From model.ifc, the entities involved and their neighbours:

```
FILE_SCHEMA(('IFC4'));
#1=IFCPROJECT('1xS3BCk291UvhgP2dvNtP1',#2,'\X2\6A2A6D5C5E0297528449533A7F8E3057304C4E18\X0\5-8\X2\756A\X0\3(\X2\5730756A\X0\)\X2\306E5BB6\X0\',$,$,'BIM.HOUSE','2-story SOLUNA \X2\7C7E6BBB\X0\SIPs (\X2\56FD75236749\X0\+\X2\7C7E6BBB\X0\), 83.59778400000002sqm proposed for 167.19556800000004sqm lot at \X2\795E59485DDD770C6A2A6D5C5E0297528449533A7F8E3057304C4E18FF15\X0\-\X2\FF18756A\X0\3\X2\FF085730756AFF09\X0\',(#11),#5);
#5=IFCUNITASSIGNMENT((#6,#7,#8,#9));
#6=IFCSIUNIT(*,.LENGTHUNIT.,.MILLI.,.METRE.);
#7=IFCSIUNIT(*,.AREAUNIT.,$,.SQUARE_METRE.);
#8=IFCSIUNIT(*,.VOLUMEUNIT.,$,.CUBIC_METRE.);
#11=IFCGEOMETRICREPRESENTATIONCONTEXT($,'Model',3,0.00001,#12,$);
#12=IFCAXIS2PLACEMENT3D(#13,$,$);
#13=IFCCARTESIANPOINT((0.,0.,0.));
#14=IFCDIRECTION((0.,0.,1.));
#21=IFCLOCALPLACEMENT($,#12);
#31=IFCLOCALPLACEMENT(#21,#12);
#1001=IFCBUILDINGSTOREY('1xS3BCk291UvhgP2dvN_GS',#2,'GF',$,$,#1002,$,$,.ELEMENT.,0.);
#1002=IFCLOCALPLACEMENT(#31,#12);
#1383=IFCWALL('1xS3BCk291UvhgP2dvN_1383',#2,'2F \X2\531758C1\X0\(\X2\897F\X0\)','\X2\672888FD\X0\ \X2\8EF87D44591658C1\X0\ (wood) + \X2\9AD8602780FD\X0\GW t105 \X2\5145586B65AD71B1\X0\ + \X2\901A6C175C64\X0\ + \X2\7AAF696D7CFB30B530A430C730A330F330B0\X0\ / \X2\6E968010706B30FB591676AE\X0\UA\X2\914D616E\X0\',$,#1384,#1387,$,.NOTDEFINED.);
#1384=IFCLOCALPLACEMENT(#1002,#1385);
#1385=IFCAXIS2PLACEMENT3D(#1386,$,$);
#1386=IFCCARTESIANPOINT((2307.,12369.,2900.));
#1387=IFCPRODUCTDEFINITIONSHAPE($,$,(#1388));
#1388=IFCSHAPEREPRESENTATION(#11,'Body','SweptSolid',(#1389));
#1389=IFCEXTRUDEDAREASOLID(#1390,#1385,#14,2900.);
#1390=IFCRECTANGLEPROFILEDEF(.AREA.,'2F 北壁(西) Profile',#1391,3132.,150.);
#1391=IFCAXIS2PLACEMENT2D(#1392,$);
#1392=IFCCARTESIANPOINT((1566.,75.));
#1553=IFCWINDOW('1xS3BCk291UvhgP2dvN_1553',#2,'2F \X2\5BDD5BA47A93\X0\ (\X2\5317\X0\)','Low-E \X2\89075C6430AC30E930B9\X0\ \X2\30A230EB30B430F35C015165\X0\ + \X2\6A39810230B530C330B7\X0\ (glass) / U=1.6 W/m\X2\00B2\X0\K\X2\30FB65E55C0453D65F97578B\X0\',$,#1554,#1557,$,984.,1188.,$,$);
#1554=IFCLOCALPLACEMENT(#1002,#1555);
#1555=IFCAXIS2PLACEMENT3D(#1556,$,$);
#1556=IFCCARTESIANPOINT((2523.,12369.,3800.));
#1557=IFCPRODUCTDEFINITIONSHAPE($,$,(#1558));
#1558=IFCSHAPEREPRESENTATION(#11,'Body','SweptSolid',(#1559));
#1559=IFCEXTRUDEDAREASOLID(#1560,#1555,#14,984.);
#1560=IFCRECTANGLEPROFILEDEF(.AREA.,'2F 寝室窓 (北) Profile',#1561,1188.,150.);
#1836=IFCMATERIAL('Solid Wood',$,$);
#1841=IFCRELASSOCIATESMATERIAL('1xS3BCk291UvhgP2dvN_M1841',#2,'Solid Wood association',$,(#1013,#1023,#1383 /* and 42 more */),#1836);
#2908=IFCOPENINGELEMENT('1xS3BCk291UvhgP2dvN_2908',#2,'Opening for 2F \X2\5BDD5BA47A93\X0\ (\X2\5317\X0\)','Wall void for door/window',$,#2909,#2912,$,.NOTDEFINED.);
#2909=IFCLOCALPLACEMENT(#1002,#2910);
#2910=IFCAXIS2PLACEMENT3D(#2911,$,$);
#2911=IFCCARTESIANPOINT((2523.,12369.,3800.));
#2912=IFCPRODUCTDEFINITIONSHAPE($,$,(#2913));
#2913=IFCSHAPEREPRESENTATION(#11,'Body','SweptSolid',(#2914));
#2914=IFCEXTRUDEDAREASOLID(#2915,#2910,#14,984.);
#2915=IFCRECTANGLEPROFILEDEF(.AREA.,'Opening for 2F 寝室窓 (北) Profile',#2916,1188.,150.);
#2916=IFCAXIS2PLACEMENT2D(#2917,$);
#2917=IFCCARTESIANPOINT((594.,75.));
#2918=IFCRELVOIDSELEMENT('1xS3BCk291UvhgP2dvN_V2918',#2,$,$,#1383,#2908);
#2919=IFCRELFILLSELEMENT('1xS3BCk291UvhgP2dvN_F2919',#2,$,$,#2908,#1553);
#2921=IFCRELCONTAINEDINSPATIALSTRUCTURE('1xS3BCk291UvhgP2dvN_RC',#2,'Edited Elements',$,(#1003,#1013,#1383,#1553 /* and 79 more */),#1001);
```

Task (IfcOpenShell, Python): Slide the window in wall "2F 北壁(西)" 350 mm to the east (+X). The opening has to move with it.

```python
import ifcopenshell
import ifcopenshell.api.geometry
import ifcopenshell.util.placement

model = ifcopenshell.open("model.ifc")

window = model.by_guid("1xS3BCk291UvhgP2dvN_1553")
opening = window.FillsVoids[0].RelatingOpeningElement
wall = opening.VoidsElements[0].RelatingBuildingElement

wall_matrix = ifcopenshell.util.placement.get_local_placement(wall.ObjectPlacement)
shift = wall_matrix[:3, 0] * 350.0
before = ifcopenshell.util.placement.get_local_placement(window.ObjectPlacement)[:3, 3].copy()

# The window is not placed relative to its opening, so move both.
for product in (opening, window):
    matrix = ifcopenshell.util.placement.get_local_placement(product.ObjectPlacement)
    matrix[:3, 3] += shift
    ifcopenshell.api.geometry.edit_object_placement(model, product=product, matrix=matrix, is_si=False)

after = ifcopenshell.util.placement.get_local_placement(window.ObjectPlacement)[:3, 3]
print("window moved by", (after - before).round(3) + 0.0)

model.write("model-out.ifc")
```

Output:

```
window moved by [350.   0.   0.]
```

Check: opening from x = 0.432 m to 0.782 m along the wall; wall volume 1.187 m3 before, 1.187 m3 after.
